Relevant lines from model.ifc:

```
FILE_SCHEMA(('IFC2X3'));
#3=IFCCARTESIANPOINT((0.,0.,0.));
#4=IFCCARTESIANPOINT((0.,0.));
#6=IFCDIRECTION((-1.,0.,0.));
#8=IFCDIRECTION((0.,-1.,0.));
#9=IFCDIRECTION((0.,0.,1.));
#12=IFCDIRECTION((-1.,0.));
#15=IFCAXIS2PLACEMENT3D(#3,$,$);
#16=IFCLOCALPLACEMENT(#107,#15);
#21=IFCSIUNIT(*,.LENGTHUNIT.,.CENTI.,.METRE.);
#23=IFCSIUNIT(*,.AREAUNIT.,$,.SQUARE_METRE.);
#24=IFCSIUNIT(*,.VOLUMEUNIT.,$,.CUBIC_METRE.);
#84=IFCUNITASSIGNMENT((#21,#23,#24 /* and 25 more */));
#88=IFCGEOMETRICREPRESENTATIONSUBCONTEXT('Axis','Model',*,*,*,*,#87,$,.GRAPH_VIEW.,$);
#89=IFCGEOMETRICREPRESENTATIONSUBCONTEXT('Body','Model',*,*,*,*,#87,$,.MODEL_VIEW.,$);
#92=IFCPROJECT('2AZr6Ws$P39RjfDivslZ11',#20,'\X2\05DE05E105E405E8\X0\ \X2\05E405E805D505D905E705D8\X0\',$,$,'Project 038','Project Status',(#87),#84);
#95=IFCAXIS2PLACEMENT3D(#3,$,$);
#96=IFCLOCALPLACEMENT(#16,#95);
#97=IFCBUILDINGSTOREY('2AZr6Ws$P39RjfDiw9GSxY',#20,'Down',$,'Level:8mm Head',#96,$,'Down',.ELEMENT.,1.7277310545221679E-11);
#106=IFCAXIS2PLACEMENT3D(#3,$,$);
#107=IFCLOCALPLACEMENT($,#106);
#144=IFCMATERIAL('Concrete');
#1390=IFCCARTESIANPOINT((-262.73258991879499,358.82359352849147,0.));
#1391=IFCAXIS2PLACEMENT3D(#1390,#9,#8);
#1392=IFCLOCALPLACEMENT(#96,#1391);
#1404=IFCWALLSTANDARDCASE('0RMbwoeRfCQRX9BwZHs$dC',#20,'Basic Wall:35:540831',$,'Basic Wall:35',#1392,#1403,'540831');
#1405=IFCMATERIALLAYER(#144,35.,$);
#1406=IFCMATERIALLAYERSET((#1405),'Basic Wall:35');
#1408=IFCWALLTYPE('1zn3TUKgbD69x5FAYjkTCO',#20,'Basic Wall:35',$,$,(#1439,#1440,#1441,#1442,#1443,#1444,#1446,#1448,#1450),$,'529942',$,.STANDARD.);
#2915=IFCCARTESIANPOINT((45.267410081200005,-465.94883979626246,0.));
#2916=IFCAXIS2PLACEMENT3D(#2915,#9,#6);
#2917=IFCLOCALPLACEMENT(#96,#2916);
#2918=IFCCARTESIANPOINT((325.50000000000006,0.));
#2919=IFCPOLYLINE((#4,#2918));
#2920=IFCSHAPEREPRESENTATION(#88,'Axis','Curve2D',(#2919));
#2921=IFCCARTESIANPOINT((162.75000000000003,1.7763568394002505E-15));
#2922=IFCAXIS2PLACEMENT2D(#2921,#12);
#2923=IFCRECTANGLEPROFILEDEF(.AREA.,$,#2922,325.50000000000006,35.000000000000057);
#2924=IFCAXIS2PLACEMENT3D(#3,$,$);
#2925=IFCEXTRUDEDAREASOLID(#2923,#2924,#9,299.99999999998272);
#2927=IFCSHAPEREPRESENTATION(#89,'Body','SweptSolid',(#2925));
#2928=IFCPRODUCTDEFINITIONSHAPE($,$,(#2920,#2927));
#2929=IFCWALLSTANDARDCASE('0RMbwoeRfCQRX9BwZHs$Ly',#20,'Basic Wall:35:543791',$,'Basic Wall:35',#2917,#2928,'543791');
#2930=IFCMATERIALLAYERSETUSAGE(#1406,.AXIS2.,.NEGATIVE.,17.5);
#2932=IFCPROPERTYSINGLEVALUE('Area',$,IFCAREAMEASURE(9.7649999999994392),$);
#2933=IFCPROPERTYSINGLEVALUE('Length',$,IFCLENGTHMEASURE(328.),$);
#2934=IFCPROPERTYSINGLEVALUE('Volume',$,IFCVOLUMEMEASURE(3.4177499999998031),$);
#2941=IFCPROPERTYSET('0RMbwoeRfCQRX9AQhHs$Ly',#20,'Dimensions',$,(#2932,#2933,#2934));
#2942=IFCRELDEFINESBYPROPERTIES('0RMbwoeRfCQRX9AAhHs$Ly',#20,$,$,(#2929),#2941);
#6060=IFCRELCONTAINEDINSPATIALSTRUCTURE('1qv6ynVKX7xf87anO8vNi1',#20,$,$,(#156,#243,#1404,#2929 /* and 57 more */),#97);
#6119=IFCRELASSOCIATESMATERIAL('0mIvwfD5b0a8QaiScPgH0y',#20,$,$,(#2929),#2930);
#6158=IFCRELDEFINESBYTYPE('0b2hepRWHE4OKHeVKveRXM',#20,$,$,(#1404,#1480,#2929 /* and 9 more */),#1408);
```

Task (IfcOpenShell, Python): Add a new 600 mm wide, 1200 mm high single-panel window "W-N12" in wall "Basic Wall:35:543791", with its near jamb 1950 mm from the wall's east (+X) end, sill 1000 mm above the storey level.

```python
import numpy as np
import ifcopenshell
import ifcopenshell.api.feature
import ifcopenshell.api.geometry
import ifcopenshell.api.pset
import ifcopenshell.api.root
import ifcopenshell.api.spatial
import ifcopenshell.api.type
import ifcopenshell.geom
import ifcopenshell.util.element
import ifcopenshell.util.placement
import ifcopenshell.util.representation
import ifcopenshell.util.shape
import ifcopenshell.util.unit

model = ifcopenshell.open("model.ifc")
unit_scale = ifcopenshell.util.unit.calculate_unit_scale(model)
area_scale = ifcopenshell.util.unit.calculate_unit_scale(model, "AREAUNIT")
volume_scale = ifcopenshell.util.unit.calculate_unit_scale(model, "VOLUMEUNIT")
settings = ifcopenshell.geom.settings()


def volume(element):
    """Net volume in cubic metres, openings subtracted."""
    shape = ifcopenshell.geom.create_shape(settings, element)
    return ifcopenshell.util.shape.get_volume(shape.geometry)


wall = model.by_guid("0RMbwoeRfCQRX9BwZHs$Ly")
storey = ifcopenshell.util.element.get_container(wall, ifc_class="IfcBuildingStorey")
context = ifcopenshell.util.representation.get_context(model, "Model", "Body", "MODEL_VIEW")
before = volume(wall)

width, height, from_end, sill = 0.6, 1.2, 1.95, 1  # metres

# The wall runs along its own X axis, and the end named is its -X end.
wall_shape = ifcopenshell.geom.create_shape(settings, wall)
x, y, z = ifcopenshell.util.shape.get_vertices(wall_shape.geometry).T
start = x.min() + from_end
face, thickness = float(y.min()), float(y.max() - y.min())
wall_matrix = ifcopenshell.util.placement.get_local_placement(wall.ObjectPlacement)
level = ifcopenshell.util.placement.get_local_placement(storey.ObjectPlacement)[2, 3]


def in_wall(x, y):
    """Placement at x, y metres in the wall's axes, at sill height."""
    matrix = wall_matrix.copy()
    matrix[:, 3] = wall_matrix @ np.array([x / unit_scale, y / unit_scale, 0.0, 1.0])
    matrix[2, 3] = level + sill / unit_scale
    return matrix


# Opening: a box that overshoots both wall faces by 50 mm.
opening = ifcopenshell.api.root.create_entity(model, ifc_class="IfcOpeningElement")
box = ifcopenshell.api.geometry.add_wall_representation(
    model, context=context, length=width, height=height, thickness=thickness + 0.1
)
ifcopenshell.api.geometry.assign_representation(model, product=opening, representation=box)
ifcopenshell.api.geometry.edit_object_placement(model, product=opening, matrix=in_wall(start, face - 0.05), is_si=False)
ifcopenshell.api.feature.add_feature(model, feature=opening, element=wall)

window = ifcopenshell.api.root.create_entity(model, ifc_class="IfcWindow", name="W-N12")
window.OverallWidth, window.OverallHeight = width / unit_scale, height / unit_scale
body = ifcopenshell.api.geometry.add_window_representation(
    model,
    context=context,
    overall_width=window.OverallWidth,
    overall_height=window.OverallHeight,
    partition_type="SINGLE_PANEL",
)
ifcopenshell.api.geometry.assign_representation(model, product=window, representation=body)
ifcopenshell.api.spatial.assign_container(model, products=[window], relating_structure=storey)
fills = ifcopenshell.api.feature.add_filling(model, opening=opening, element=window)
fills.OwnerHistory = window.OwnerHistory  # required in IFC2X3

# IFC2X3 keeps the operation on the window style.
style = ifcopenshell.api.root.create_entity(model, ifc_class="IfcWindowStyle", name="W-N12")
style.OperationType, style.ConstructionType = "SINGLE_PANEL", "NOTDEFINED"
style.ParameterTakesPrecedence = style.Sizeable = False
ifcopenshell.api.type.assign_type(model, related_objects=[window], relating_type=style)

# Centre the window in the wall's thickness.
ifcopenshell.api.geometry.edit_object_placement(model, product=window, matrix=in_wall(start, face), is_si=False)
window_shape = ifcopenshell.geom.create_shape(settings, window)
depth = ifcopenshell.util.shape.get_vertices(window_shape.geometry)[:, 1]
offset = face + thickness / 2 - (depth.min() + depth.max()) / 2
ifcopenshell.api.geometry.edit_object_placement(model, product=window, matrix=in_wall(start, offset), is_si=False)

after = volume(wall)

# Update the wall's stored quantities.
pset = model.by_id(ifcopenshell.util.element.get_pset(wall, "Dimensions", should_inherit=False)["id"])
ifcopenshell.api.pset.edit_pset(model, pset=pset, properties={
    "Area": model.create_entity("IfcAreaMeasure", after / thickness / area_scale),
    "Volume": model.create_entity("IfcVolumeMeasure", after / volume_scale),
})

print(f"wall volume {before:.3f} -> {after:.3f} m3")

model.write("model_rev.ifc")
```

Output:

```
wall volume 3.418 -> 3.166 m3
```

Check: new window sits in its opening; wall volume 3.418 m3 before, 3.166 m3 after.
